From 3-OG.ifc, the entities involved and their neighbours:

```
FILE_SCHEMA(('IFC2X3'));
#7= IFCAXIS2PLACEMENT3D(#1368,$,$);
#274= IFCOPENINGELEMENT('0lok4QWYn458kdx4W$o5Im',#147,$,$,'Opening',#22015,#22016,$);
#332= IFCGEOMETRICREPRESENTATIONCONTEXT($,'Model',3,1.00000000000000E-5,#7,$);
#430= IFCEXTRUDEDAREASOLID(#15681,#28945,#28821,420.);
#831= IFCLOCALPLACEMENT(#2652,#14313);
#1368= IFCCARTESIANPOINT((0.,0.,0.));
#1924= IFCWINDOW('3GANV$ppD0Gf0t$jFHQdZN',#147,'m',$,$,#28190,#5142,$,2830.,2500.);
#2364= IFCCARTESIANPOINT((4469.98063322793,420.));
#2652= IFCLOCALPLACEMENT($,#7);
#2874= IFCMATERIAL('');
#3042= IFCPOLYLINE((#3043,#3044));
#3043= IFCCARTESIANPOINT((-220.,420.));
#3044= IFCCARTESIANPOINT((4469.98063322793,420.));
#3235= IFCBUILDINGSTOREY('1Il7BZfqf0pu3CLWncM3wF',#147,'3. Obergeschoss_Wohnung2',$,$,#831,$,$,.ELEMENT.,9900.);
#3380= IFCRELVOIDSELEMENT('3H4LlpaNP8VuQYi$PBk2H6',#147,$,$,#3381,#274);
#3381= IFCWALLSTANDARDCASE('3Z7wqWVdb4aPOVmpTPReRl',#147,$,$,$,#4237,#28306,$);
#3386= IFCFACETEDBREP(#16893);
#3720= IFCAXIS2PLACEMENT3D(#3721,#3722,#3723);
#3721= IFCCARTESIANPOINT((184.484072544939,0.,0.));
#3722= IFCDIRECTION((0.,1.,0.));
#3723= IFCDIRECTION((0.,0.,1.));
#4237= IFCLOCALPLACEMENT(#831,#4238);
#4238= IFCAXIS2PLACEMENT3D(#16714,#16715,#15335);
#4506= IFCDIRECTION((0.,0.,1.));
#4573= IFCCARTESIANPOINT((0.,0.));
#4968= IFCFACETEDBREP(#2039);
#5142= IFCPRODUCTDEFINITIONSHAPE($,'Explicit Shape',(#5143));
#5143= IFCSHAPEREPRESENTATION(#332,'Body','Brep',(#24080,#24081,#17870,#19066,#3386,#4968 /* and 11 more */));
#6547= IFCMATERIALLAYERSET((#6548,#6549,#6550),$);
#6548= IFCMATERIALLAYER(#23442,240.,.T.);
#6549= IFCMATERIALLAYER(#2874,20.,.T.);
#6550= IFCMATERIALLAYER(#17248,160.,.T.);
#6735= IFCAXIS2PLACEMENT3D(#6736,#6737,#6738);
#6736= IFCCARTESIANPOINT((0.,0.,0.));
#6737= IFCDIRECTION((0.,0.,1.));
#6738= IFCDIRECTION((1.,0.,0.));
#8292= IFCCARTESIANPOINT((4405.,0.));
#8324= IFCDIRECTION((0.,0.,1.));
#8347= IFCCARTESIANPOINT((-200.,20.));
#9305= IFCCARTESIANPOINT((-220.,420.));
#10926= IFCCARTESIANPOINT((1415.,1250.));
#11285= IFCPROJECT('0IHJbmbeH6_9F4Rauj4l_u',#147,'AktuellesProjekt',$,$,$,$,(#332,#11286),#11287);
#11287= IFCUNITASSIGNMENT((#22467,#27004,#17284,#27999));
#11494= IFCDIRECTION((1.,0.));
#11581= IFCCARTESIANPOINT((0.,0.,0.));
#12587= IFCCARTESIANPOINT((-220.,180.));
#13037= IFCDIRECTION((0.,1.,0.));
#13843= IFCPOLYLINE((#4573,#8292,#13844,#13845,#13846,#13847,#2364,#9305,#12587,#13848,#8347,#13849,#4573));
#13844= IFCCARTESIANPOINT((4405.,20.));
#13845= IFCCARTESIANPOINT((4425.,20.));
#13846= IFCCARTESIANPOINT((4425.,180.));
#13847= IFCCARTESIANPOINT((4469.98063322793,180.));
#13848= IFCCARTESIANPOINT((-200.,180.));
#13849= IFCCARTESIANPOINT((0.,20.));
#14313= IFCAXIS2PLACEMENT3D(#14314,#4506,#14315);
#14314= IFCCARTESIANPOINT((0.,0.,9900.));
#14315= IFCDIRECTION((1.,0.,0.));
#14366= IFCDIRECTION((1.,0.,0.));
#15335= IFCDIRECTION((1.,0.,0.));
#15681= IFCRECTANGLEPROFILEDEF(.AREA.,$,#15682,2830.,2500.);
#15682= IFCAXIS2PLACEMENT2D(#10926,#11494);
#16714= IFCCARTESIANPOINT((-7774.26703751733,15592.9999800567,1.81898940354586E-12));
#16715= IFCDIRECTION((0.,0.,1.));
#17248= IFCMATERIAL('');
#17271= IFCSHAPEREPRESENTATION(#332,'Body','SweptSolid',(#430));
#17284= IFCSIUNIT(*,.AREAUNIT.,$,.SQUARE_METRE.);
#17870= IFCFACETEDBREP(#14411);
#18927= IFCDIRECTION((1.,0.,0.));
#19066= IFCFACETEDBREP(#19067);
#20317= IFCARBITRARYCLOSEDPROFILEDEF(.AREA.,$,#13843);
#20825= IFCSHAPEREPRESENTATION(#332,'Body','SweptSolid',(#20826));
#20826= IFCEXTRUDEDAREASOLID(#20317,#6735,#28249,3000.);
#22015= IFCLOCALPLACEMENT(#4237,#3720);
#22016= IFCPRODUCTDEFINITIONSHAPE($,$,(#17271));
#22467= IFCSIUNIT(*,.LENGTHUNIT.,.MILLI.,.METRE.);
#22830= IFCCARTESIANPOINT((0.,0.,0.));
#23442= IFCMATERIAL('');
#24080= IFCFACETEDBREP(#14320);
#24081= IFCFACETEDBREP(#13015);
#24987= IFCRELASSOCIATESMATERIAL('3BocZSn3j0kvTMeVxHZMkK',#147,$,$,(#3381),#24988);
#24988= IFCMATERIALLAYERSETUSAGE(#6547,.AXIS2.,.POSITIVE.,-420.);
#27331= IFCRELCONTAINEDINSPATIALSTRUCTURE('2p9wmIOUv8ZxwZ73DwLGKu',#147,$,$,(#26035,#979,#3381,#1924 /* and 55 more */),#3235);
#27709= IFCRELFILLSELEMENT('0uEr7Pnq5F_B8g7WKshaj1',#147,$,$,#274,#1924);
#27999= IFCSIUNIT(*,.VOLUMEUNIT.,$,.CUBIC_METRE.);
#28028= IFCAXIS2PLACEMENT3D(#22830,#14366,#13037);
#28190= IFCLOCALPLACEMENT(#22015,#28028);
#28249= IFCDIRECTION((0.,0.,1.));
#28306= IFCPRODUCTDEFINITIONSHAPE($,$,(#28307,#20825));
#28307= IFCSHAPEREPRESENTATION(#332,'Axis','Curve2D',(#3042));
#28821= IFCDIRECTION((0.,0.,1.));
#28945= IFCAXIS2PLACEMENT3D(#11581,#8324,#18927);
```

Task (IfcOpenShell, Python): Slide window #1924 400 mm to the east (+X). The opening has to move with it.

```python
import ifcopenshell
import ifcopenshell.api.geometry
import ifcopenshell.util.placement
import ifcopenshell.util.unit

model = ifcopenshell.open("3-OG.ifc")
unit_scale = ifcopenshell.util.unit.calculate_unit_scale(model)

window = model.by_guid("3GANV$ppD0Gf0t$jFHQdZN")
opening = window.FillsVoids[0].RelatingOpeningElement
wall = opening.VoidsElements[0].RelatingBuildingElement

wall_matrix = ifcopenshell.util.placement.get_local_placement(wall.ObjectPlacement)
shift = wall_matrix[:3, 0] * 0.4 / unit_scale
before = ifcopenshell.util.placement.get_local_placement(window.ObjectPlacement)[:3, 3].copy()

# The window is placed relative to its opening, so it follows when the opening moves.
matrix = ifcopenshell.util.placement.get_local_placement(opening.ObjectPlacement)
matrix[:3, 3] += shift
ifcopenshell.api.geometry.edit_object_placement(
    model, product=opening, matrix=matrix, is_si=False, should_transform_children=True
)

after = ifcopenshell.util.placement.get_local_placement(window.ObjectPlacement)[:3, 3]
print("window moved by", (after - before).round(3) + 0.0)

model.write("3-OG_edited.ifc")
```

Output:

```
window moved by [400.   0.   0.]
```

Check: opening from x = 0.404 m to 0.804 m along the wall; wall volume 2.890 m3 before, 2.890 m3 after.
